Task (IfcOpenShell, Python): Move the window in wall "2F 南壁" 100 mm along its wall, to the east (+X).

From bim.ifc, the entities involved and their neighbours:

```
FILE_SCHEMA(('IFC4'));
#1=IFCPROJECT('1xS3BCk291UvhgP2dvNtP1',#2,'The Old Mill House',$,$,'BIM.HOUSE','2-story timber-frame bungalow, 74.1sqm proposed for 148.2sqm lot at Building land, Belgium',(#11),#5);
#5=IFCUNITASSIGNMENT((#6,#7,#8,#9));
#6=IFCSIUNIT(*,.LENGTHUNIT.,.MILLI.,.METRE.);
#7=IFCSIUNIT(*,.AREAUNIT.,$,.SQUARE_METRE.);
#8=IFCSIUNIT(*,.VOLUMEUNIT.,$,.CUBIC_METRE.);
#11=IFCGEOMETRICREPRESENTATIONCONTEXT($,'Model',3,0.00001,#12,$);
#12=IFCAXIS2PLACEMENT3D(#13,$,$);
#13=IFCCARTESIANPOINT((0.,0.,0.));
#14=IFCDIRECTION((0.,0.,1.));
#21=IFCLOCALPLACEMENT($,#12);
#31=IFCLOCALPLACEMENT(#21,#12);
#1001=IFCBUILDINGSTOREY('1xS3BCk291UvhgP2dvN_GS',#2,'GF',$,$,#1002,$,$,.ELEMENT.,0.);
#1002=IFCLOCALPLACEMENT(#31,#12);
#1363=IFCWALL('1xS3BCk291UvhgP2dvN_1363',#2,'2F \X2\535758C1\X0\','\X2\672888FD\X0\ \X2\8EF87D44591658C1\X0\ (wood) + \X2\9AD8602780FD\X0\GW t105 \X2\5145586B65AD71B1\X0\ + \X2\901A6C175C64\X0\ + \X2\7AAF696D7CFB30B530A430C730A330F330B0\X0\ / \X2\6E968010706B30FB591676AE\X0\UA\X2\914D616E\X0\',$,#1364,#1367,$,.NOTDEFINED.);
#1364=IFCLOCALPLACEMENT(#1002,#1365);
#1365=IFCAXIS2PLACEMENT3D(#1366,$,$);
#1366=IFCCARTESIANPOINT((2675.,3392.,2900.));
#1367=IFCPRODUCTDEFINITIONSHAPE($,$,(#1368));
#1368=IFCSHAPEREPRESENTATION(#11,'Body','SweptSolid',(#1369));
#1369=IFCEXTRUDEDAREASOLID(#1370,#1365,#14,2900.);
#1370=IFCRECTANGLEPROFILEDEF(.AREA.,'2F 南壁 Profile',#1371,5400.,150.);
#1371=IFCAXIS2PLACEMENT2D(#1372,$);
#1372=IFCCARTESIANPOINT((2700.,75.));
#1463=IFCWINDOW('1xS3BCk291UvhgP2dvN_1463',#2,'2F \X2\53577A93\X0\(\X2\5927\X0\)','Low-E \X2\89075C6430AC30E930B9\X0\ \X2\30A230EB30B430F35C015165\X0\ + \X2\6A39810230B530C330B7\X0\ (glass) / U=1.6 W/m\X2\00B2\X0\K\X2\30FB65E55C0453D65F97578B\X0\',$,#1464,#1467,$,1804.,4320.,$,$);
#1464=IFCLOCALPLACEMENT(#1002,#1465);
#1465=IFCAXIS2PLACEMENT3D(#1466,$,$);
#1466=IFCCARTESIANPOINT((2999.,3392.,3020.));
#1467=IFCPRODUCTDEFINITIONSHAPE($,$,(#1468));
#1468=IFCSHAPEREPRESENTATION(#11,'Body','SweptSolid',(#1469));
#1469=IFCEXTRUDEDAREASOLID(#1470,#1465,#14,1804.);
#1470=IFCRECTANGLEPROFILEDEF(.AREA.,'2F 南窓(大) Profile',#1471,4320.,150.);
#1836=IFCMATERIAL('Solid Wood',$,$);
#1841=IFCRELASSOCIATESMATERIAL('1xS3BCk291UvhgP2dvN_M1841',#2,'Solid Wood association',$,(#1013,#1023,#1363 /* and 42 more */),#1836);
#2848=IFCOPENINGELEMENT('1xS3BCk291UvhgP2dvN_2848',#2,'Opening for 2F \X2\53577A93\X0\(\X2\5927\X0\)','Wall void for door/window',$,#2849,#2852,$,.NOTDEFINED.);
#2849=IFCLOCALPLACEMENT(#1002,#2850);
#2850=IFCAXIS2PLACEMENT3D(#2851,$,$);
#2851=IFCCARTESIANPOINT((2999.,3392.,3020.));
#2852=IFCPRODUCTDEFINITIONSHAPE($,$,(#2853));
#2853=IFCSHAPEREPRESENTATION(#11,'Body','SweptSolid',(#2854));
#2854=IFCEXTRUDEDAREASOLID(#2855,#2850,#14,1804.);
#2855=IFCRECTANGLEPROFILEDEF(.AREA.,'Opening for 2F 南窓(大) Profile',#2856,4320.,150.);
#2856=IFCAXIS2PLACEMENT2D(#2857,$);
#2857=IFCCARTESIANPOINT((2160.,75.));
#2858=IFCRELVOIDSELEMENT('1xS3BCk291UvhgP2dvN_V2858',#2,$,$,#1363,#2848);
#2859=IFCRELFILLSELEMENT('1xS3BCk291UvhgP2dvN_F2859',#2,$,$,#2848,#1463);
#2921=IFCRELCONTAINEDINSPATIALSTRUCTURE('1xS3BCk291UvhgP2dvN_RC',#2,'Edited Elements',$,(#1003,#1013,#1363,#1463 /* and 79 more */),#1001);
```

```python
import ifcopenshell
import ifcopenshell.api.geometry
import ifcopenshell.util.placement

model = ifcopenshell.open("bim.ifc")

window = model.by_guid("1xS3BCk291UvhgP2dvN_1463")
opening = window.FillsVoids[0].RelatingOpeningElement
wall = opening.VoidsElements[0].RelatingBuildingElement

wall_matrix = ifcopenshell.util.placement.get_local_placement(wall.ObjectPlacement)
shift = wall_matrix[:3, 0] * 100.0
before = ifcopenshell.util.placement.get_local_placement(window.ObjectPlacement)[:3, 3].copy()

# The window is not placed relative to its opening, so move both.
for product in (opening, window):
    matrix = ifcopenshell.util.placement.get_local_placement(product.ObjectPlacement)
    matrix[:3, 3] += shift
    ifcopenshell.api.geometry.edit_object_placement(model, product=product, matrix=matrix, is_si=False)

after = ifcopenshell.util.placement.get_local_placement(window.ObjectPlacement)[:3, 3]
print("window moved by", (after - before).round(3) + 0.0)

model.write("bim_v2.ifc")
```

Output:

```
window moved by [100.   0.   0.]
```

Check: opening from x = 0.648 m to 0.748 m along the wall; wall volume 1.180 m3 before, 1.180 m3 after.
